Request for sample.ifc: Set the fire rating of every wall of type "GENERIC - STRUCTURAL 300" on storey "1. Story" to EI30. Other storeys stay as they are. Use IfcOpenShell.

First a look at what the model holds.

```python
import ifcopenshell
import ifcopenshell.util.element

model = ifcopenshell.open("sample.ifc")
print(model.schema)
storey = next(s for s in model.by_type("IfcBuildingStorey") if s.Name == "1. Story")
walls = [e for e in ifcopenshell.util.element.get_decomposition(storey) if e.is_a("IfcWall")]
seen = {}
for e in walls:
    element_type = ifcopenshell.util.element.get_type(e)
    key = (element_type.Name if element_type != e and element_type else None, ifcopenshell.util.element.get_pset(e, "Pset_WallCommon", "FireRating"))
    seen[key] = seen.get(key, 0) + 1
for (name, value), count in sorted(seen.items(), key=str):
    print(count, "x", name, "|", value)
```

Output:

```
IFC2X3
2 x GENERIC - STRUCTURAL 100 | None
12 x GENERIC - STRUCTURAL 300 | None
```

```python
import ifcopenshell
import ifcopenshell.api.pset
import ifcopenshell.util.element

model = ifcopenshell.open("sample.ifc")

storey = next(s for s in model.by_type("IfcBuildingStorey") if s.Name == "1. Story")
walls = [e for e in ifcopenshell.util.element.get_decomposition(storey) if e.is_a("IfcWall")]

count = 0
for e in walls:
    element_type = ifcopenshell.util.element.get_type(e)
    if element_type in (None, e) or element_type.Name != "GENERIC - STRUCTURAL 300":
        continue
    # add_pset returns the element's existing set when there is one.
    pset = ifcopenshell.api.pset.add_pset(model, product=e, name="Pset_WallCommon")
    ifcopenshell.api.pset.edit_pset(model, pset=pset, properties={"FireRating": "EI30"})
    count += 1

print(count, "walls updated")

model.write("sample_v2.ifc")
```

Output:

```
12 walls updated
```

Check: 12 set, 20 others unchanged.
